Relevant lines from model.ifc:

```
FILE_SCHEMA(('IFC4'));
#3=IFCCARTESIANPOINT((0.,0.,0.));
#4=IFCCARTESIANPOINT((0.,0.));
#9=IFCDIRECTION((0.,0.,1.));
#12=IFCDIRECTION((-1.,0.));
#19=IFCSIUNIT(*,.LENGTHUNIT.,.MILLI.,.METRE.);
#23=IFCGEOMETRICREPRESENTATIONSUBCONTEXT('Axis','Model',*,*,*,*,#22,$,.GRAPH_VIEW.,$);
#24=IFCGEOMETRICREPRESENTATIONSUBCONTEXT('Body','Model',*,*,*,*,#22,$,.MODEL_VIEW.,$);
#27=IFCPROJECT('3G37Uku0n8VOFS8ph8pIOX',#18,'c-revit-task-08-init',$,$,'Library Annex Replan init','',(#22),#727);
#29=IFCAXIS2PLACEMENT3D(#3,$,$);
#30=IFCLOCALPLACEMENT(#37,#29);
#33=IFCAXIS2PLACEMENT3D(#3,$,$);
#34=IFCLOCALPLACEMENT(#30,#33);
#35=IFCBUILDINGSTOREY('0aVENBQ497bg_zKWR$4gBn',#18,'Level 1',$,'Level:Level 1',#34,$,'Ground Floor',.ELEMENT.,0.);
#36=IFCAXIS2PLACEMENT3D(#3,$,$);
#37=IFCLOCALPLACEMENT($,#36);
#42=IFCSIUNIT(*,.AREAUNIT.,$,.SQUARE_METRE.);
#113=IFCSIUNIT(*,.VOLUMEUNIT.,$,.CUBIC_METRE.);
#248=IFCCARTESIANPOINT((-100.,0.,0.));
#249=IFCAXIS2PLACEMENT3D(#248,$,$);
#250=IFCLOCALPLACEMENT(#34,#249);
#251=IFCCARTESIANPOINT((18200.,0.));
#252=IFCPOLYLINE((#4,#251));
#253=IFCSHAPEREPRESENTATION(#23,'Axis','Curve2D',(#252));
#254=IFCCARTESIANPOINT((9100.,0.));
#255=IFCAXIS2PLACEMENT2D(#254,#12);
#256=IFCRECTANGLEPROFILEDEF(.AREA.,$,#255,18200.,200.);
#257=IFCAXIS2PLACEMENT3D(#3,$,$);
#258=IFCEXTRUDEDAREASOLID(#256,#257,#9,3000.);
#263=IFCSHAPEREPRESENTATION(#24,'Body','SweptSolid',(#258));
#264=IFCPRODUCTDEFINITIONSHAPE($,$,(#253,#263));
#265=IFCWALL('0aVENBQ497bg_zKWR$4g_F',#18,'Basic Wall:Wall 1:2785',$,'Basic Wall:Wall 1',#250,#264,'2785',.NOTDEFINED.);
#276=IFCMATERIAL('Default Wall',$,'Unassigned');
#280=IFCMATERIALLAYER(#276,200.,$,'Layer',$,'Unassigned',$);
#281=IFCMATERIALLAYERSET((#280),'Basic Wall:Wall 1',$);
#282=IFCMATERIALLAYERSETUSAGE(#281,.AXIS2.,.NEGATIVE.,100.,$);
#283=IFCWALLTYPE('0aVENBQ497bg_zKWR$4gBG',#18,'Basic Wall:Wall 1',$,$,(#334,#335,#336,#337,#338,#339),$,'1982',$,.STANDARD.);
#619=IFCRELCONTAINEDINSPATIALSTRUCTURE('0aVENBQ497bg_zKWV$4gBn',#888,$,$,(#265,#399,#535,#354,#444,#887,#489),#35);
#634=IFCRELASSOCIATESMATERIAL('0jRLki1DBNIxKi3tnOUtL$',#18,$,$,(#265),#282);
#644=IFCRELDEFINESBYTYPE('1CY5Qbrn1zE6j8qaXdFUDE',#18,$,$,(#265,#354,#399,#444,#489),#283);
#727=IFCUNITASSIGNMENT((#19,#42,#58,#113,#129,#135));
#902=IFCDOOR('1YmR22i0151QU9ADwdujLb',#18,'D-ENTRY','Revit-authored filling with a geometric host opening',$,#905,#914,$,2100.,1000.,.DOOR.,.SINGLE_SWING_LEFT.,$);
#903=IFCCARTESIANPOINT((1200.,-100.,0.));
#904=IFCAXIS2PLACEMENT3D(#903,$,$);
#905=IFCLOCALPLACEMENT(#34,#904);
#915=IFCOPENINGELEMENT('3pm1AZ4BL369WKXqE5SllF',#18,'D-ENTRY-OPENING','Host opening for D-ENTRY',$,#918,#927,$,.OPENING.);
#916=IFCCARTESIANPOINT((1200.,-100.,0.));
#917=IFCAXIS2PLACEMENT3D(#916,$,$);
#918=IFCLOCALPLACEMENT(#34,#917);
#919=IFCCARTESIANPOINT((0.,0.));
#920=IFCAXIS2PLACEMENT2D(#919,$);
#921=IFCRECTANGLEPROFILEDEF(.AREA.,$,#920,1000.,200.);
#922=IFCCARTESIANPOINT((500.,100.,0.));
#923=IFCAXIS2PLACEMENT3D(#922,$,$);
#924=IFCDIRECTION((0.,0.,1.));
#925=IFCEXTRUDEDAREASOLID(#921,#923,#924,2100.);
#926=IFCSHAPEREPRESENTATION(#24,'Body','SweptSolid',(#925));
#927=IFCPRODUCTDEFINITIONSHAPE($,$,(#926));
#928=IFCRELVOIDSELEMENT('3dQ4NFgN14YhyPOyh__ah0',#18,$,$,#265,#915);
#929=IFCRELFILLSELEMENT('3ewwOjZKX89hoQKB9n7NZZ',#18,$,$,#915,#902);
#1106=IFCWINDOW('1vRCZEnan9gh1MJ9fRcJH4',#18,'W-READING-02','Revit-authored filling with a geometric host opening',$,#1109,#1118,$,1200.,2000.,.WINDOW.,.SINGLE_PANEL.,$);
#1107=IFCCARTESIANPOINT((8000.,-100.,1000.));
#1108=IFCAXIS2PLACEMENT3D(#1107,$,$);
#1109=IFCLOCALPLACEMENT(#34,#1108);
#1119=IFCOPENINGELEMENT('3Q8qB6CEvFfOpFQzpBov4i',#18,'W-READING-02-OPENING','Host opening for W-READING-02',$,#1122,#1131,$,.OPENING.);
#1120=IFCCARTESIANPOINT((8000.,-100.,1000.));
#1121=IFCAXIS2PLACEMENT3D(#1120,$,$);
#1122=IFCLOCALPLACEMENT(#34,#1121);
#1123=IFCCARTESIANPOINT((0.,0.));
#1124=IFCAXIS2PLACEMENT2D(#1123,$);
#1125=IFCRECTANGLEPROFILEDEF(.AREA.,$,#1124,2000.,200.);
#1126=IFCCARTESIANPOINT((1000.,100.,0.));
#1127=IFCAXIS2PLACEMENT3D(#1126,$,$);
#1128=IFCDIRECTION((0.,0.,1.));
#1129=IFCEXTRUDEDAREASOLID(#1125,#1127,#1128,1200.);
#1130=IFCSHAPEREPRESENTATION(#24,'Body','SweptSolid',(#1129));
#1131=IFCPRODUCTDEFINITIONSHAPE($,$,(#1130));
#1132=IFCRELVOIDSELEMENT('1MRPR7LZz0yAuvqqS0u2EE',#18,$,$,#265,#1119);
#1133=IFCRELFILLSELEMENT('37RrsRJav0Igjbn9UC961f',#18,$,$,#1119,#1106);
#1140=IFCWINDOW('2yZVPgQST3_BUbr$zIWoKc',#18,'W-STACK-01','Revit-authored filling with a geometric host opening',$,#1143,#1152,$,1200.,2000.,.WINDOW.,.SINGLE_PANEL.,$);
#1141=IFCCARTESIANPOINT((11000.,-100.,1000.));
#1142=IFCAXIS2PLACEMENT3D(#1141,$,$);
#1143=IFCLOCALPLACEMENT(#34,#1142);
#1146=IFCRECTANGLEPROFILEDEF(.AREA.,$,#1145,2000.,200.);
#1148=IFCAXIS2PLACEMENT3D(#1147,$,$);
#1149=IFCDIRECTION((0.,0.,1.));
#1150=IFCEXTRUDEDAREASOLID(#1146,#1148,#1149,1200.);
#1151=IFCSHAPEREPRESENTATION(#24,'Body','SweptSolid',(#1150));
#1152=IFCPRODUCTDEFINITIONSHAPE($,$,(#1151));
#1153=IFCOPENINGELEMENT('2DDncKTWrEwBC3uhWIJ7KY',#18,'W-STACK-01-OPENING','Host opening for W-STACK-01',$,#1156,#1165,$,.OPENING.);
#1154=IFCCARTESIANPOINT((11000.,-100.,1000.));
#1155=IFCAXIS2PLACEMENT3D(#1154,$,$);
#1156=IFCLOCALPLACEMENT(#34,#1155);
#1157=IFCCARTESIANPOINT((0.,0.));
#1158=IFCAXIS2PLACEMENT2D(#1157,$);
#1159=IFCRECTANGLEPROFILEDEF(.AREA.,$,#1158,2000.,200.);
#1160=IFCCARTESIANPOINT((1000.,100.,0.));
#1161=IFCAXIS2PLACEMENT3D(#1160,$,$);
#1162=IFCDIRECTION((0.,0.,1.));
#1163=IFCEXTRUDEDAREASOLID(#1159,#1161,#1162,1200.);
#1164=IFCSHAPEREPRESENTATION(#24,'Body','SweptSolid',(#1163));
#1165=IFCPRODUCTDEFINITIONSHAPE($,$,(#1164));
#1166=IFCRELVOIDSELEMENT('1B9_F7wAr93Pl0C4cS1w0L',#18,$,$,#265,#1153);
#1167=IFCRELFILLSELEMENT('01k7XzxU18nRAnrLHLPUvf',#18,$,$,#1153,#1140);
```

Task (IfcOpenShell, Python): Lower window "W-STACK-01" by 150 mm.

```python
import numpy as np
import ifcopenshell
import ifcopenshell.api.geometry
import ifcopenshell.util.placement
import ifcopenshell.util.unit

model = ifcopenshell.open("model.ifc")
unit_scale = ifcopenshell.util.unit.calculate_unit_scale(model)

window = model.by_guid("2yZVPgQST3_BUbr$zIWoKc")
opening = window.FillsVoids[0].RelatingOpeningElement
dz = -0.15 / unit_scale

shift = np.array([0.0, 0.0, dz])
# The window is not placed relative to its opening, so move both.
for product in (opening, window):
    matrix = ifcopenshell.util.placement.get_local_placement(product.ObjectPlacement)
    matrix[:3, 3] += shift
    ifcopenshell.api.geometry.edit_object_placement(model, product=product, matrix=matrix, is_si=False)

print(f"moved by {dz * unit_scale:+.3f} m")

model.write("model_updated.ifc")
```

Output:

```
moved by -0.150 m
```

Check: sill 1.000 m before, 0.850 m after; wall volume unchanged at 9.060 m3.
